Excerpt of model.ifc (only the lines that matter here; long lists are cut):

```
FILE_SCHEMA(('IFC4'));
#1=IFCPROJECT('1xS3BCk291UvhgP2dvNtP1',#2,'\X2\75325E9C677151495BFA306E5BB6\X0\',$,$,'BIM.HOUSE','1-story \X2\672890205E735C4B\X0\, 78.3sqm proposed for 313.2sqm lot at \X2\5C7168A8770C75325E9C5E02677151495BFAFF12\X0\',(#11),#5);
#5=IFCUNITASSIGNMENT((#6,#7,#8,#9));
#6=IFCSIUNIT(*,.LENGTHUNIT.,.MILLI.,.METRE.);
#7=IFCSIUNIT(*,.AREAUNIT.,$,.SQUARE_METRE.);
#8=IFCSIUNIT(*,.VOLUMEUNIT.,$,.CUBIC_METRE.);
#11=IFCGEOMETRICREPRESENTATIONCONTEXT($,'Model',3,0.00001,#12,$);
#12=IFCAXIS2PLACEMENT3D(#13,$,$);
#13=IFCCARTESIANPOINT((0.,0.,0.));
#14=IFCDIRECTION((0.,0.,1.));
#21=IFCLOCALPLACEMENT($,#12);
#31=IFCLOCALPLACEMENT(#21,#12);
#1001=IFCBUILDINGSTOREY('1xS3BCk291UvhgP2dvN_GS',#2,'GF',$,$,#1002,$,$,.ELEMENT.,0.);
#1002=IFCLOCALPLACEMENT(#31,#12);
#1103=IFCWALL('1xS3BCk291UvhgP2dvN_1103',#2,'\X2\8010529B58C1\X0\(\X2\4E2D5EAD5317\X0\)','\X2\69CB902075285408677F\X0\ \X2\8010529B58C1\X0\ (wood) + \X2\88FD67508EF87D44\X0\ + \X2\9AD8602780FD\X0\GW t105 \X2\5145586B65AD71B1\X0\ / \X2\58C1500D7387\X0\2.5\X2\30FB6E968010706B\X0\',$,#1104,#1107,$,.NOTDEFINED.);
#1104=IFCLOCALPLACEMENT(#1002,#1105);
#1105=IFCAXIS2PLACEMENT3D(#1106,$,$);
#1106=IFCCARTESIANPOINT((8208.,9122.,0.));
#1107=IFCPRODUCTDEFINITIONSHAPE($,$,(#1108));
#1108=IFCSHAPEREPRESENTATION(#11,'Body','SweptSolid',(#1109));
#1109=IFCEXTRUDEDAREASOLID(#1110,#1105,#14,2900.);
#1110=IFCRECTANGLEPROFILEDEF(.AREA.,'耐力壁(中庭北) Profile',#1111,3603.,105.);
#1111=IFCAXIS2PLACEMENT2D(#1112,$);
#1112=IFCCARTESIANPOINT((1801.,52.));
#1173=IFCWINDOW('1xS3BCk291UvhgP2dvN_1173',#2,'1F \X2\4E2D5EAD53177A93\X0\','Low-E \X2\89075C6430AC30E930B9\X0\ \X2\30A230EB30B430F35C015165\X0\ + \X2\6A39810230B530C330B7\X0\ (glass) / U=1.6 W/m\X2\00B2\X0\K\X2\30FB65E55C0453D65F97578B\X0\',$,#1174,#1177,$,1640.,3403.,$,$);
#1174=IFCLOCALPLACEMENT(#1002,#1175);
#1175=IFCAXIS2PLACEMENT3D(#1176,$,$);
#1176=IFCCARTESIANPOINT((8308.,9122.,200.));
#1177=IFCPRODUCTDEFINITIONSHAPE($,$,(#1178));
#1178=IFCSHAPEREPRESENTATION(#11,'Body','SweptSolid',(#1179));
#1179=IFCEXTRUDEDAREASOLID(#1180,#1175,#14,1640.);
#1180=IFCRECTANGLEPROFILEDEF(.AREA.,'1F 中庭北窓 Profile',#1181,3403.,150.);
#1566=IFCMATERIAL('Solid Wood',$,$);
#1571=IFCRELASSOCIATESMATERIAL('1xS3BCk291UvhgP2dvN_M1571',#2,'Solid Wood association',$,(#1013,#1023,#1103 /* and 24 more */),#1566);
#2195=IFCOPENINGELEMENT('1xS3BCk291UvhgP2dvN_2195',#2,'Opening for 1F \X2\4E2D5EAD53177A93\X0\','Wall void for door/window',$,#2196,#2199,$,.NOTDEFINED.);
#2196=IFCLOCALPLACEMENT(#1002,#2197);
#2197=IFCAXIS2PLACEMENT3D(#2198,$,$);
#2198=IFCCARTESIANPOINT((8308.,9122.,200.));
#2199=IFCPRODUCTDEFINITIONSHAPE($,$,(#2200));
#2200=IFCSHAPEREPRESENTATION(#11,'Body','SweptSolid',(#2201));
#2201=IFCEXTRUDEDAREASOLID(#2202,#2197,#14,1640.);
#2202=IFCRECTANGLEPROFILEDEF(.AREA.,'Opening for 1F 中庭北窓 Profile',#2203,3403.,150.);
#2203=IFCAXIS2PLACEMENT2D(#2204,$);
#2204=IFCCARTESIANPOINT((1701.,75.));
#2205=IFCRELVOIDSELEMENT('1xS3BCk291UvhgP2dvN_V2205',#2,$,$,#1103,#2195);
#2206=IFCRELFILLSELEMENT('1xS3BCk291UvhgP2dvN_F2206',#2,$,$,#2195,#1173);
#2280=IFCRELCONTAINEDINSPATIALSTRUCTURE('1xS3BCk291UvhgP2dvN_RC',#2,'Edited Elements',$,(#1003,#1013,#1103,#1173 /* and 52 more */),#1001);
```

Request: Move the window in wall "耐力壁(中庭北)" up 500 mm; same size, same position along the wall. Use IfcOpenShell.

```python
import numpy as np
import ifcopenshell
import ifcopenshell.api.geometry
import ifcopenshell.util.placement
import ifcopenshell.util.unit

model = ifcopenshell.open("model.ifc")
unit_scale = ifcopenshell.util.unit.calculate_unit_scale(model)

window = model.by_guid("1xS3BCk291UvhgP2dvN_1173")
opening = window.FillsVoids[0].RelatingOpeningElement
dz = 500.0

shift = np.array([0.0, 0.0, dz])
# The window is not placed relative to its opening, so move both.
for product in (opening, window):
    matrix = ifcopenshell.util.placement.get_local_placement(product.ObjectPlacement)
    matrix[:3, 3] += shift
    ifcopenshell.api.geometry.edit_object_placement(model, product=product, matrix=matrix, is_si=False)

print(f"moved by {dz * unit_scale:+.3f} m")

model.write("model-out.ifc")
```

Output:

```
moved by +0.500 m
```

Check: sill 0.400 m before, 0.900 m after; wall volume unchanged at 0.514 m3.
